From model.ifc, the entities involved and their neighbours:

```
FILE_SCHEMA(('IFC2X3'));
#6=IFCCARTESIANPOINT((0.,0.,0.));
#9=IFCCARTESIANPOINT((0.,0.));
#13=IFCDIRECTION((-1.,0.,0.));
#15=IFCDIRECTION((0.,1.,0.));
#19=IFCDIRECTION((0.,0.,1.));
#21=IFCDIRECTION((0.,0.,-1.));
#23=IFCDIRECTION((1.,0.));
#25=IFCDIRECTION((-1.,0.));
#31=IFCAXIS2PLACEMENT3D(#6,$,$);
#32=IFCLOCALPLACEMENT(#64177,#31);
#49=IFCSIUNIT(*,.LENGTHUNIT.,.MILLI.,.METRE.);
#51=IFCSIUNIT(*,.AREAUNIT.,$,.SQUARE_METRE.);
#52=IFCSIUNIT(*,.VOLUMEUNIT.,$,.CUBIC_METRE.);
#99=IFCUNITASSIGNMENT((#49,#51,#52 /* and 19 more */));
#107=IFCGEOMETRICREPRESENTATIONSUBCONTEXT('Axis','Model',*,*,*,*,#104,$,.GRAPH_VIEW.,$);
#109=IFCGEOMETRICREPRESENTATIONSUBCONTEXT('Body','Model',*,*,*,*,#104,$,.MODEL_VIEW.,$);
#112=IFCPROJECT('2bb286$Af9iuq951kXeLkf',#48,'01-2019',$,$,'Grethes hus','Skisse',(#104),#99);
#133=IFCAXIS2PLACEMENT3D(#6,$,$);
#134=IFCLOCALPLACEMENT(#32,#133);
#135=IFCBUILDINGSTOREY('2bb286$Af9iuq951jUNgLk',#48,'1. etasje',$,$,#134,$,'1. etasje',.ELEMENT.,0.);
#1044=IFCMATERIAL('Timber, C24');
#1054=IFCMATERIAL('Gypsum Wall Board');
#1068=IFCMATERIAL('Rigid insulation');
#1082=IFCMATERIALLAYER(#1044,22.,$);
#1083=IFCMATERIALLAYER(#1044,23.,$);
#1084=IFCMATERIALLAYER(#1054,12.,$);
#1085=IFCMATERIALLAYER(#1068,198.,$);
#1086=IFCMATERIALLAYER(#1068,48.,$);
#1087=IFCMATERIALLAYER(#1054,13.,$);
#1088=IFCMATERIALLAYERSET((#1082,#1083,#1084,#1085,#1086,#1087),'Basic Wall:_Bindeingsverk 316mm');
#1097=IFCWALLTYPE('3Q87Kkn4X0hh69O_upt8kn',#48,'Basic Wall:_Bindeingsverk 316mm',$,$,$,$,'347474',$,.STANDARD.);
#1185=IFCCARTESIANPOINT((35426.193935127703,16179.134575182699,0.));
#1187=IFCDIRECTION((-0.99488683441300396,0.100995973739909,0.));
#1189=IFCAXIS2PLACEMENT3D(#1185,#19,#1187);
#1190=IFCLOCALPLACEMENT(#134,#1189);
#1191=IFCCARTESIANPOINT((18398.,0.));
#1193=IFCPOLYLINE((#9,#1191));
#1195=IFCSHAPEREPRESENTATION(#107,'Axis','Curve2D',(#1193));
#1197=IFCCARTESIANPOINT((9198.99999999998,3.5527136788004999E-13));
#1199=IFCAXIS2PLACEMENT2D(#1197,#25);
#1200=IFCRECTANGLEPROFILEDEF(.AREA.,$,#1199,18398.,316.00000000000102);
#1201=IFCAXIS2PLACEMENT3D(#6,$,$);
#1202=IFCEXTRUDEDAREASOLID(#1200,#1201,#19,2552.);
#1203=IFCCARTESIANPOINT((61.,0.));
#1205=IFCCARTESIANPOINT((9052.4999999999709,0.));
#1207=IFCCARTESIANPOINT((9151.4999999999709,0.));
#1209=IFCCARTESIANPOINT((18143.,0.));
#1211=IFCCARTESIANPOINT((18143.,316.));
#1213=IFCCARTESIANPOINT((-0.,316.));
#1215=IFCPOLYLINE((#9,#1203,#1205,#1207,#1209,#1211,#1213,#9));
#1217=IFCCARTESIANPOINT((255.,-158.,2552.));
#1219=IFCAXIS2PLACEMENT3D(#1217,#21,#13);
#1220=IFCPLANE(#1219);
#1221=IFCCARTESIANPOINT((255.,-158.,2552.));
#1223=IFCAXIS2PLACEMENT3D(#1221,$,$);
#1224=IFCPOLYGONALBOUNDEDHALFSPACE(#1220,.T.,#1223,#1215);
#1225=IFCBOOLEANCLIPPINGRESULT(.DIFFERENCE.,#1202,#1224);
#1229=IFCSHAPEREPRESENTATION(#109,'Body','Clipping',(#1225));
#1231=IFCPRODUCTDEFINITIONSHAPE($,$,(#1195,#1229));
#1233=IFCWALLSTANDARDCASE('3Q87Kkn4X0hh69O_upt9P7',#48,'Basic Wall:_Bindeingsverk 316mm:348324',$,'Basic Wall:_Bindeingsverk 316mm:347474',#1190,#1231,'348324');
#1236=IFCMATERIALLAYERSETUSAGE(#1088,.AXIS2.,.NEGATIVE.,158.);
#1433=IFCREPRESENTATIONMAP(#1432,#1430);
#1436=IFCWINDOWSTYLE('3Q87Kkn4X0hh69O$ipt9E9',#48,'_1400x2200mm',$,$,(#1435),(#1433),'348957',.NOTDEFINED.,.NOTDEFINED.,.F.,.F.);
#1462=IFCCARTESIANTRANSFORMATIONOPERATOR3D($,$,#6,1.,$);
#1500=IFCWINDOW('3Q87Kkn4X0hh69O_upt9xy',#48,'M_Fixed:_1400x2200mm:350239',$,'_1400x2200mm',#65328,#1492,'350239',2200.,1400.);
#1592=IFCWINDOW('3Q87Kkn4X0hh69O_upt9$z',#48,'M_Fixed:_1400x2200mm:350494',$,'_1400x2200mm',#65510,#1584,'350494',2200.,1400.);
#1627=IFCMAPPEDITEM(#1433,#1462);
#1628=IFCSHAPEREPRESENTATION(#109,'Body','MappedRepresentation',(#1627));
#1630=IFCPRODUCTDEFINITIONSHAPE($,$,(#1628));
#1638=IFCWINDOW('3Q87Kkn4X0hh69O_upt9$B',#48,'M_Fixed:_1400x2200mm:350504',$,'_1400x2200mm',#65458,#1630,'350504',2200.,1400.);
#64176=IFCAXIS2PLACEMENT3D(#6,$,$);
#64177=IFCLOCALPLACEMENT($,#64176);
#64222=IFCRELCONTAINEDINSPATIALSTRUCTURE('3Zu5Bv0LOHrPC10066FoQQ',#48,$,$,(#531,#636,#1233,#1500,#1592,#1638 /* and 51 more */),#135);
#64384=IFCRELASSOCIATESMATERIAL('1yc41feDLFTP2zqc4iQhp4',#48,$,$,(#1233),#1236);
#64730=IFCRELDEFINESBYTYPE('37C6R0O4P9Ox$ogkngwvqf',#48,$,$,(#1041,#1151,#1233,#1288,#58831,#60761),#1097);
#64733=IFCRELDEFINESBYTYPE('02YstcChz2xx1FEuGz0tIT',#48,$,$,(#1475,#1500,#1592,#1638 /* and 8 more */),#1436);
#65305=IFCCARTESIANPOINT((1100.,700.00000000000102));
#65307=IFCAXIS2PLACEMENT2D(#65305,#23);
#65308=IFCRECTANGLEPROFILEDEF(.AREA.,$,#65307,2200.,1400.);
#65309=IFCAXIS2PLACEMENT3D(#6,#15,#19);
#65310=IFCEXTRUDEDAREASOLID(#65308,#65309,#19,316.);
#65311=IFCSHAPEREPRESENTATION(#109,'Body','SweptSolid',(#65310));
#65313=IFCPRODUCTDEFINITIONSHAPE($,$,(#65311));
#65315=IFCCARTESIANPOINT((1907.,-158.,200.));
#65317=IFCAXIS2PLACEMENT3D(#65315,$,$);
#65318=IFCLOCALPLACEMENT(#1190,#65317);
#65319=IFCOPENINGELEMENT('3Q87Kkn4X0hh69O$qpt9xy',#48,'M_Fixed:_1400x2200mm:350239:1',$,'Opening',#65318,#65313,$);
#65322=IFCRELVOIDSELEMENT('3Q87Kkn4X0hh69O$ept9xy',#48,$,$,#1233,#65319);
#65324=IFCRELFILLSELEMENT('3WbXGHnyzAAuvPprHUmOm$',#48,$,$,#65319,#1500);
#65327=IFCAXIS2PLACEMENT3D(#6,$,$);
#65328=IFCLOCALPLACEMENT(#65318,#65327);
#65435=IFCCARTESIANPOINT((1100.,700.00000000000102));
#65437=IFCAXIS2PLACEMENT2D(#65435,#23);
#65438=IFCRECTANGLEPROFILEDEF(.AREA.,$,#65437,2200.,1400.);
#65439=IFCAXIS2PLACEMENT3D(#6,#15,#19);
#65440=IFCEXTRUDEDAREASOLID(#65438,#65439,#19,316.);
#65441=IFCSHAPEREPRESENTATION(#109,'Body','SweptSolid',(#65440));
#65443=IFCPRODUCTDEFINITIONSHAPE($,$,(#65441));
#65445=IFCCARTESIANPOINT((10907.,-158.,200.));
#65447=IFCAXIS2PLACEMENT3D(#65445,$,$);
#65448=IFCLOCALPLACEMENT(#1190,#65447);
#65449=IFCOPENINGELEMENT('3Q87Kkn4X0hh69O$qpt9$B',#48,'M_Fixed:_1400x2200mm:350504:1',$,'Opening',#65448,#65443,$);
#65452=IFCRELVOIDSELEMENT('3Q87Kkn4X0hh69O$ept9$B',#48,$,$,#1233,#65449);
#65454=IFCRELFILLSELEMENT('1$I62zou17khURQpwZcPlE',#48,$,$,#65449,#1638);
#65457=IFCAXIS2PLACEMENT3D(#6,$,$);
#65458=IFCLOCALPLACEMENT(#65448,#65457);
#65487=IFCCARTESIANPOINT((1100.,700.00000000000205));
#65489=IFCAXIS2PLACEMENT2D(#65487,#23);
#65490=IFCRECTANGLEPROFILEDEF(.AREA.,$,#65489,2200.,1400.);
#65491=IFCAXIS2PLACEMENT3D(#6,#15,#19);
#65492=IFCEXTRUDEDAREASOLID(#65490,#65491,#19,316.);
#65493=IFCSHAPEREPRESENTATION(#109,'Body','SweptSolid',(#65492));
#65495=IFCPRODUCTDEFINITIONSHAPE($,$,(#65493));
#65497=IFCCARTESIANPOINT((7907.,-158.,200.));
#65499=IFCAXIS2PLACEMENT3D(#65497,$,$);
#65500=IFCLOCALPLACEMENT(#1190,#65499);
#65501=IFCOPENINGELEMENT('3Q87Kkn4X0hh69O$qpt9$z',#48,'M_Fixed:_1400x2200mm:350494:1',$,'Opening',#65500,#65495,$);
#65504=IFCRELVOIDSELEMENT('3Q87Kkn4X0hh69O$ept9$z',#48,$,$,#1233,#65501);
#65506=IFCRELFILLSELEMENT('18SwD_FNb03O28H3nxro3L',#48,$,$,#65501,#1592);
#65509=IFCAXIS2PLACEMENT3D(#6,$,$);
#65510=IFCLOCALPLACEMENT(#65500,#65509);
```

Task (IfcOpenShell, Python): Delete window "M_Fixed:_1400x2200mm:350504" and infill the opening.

```python
import ifcopenshell
import ifcopenshell.api.feature
import ifcopenshell.api.root
import ifcopenshell.geom
import ifcopenshell.util.shape

model = ifcopenshell.open("model.ifc")
settings = ifcopenshell.geom.settings()


def volume(element):
    """Net volume in cubic metres, openings subtracted."""
    shape = ifcopenshell.geom.create_shape(settings, element)
    return ifcopenshell.util.shape.get_volume(shape.geometry)


window = model.by_guid("3Q87Kkn4X0hh69O_upt9$B")
opening = window.FillsVoids[0].RelatingOpeningElement
wall = opening.VoidsElements[0].RelatingBuildingElement
before = volume(wall)

ifcopenshell.api.root.remove_product(model, product=window)
ifcopenshell.api.feature.remove_feature(model, feature=opening)

after = volume(wall)

print(f"wall volume {before:.3f} -> {after:.3f} m3")

model.write("model_rev.ifc")
```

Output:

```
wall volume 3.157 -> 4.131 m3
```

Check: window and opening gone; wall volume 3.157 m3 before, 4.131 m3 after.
